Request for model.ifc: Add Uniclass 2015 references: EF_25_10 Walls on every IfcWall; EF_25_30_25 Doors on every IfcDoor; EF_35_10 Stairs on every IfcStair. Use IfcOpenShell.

First a look at what the model holds.

```python
import ifcopenshell

model = ifcopenshell.open("model.ifc")
print(model.schema)
print("classifications:", [c.Name for c in model.by_type("IfcClassification")])
for ifc_class in ("IfcDoor", "IfcRoof", "IfcStair", "IfcWall", "IfcWindow"):
    print(ifc_class, len(model.by_type(ifc_class)))
```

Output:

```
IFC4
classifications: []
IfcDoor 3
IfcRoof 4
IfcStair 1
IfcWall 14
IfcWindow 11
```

```python
import ifcopenshell
import ifcopenshell.api.classification

model = ifcopenshell.open("model.ifc")

system = ifcopenshell.api.classification.add_classification(model, classification="Uniclass 2015")

codes = {
    "IfcWall": ("EF_25_10", "Walls"),
    "IfcDoor": ("EF_25_30_25", "Doors"),
    "IfcStair": ("EF_35_10", "Stairs"),
}
for ifc_class, (code, name) in codes.items():
    products = model.by_type(ifc_class)
    ifcopenshell.api.classification.add_reference(
        model, products=products, classification=system, identification=code, name=name
    )
    print(code, len(products))

model.write("model_rev.ifc")
```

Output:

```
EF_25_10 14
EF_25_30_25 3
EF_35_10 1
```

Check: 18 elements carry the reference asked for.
